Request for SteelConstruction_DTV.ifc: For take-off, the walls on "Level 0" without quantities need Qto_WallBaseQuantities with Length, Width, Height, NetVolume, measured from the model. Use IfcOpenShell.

First a look at what the model holds.

```python
import ifcopenshell
import ifcopenshell.util.element
import ifcopenshell.util.unit

model = ifcopenshell.open("SteelConstruction_DTV.ifc")
print(model.schema)
for unit_type in ("LENGTHUNIT", "AREAUNIT", "VOLUMEUNIT"):
    print(unit_type, ifcopenshell.util.unit.calculate_unit_scale(model, unit_type))
storey = next(s for s in model.by_type("IfcBuildingStorey") if s.Name == "Level 0")
walls = [e for e in ifcopenshell.util.element.get_decomposition(storey) if e.is_a("IfcWall")]
for e in sorted(walls, key=lambda e: e.id()):
    print(e.id(), e.is_a(), e.Name, list(ifcopenshell.util.element.get_psets(e, qtos_only=True)), sep=" | ")
```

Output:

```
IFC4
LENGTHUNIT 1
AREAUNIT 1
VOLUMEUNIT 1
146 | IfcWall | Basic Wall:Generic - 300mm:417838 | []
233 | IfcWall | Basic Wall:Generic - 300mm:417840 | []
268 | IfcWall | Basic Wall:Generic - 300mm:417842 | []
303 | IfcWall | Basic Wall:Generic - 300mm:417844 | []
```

```python
import ifcopenshell
import ifcopenshell.api.pset
import ifcopenshell.geom
import ifcopenshell.util.element
import ifcopenshell.util.shape
import ifcopenshell.util.unit

model = ifcopenshell.open("SteelConstruction_DTV.ifc")
unit_scale = ifcopenshell.util.unit.calculate_unit_scale(model)
volume_scale = ifcopenshell.util.unit.calculate_unit_scale(model, "VOLUMEUNIT")
settings = ifcopenshell.geom.settings()

storey = next(s for s in model.by_type("IfcBuildingStorey") if s.Name == "Level 0")
walls = [e for e in ifcopenshell.util.element.get_decomposition(storey) if e.is_a("IfcWall")]

for e in sorted(walls, key=lambda e: e.id()):
    if ifcopenshell.util.element.get_psets(e, qtos_only=True, should_inherit=False):
        continue
    # Geometry comes back in metres, in the element's own axes.
    shape = ifcopenshell.geom.create_shape(settings, e)
    values = {
        "Length": ifcopenshell.util.shape.get_x(shape.geometry) / unit_scale,
        "Width": ifcopenshell.util.shape.get_y(shape.geometry) / unit_scale,
        "Height": ifcopenshell.util.shape.get_z(shape.geometry) / unit_scale,
        "NetVolume": ifcopenshell.util.shape.get_volume(shape.geometry) / volume_scale,
    }
    qto = ifcopenshell.api.pset.add_qto(model, product=e, name="Qto_WallBaseQuantities")
    ifcopenshell.api.pset.edit_qto(model, qto=qto, properties=values)
    print(e.id(), {k: round(v, 3) for k, v in values.items()})

model.write("SteelConstruction_DTV_rev.ifc")
```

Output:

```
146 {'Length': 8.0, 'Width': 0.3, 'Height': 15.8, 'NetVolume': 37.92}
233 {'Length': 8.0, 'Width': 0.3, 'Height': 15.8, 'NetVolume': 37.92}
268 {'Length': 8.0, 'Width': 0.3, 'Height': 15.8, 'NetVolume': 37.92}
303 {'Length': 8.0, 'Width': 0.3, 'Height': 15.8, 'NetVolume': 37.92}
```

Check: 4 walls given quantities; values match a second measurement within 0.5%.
